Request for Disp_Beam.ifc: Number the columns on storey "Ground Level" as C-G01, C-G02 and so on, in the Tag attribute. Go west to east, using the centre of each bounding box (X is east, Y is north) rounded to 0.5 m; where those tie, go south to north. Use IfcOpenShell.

First a look at what the model holds.

```python
import ifcopenshell
import ifcopenshell.util.element
import ifcopenshell.util.placement

model = ifcopenshell.open("Disp_Beam.ifc")
print(model.schema)
storey = next(s for s in model.by_type("IfcBuildingStorey") if s.Name == "Ground Level")
columns = [e for e in ifcopenshell.util.element.get_decomposition(storey) if e.is_a("IfcColumn")]
for e in sorted(columns, key=lambda e: e.id()):
    origin = ifcopenshell.util.placement.get_local_placement(e.ObjectPlacement)[:3, 3]
    print(e.id(), e.Tag, e.Name, origin.round(2) + 0.0, sep=" | ")
```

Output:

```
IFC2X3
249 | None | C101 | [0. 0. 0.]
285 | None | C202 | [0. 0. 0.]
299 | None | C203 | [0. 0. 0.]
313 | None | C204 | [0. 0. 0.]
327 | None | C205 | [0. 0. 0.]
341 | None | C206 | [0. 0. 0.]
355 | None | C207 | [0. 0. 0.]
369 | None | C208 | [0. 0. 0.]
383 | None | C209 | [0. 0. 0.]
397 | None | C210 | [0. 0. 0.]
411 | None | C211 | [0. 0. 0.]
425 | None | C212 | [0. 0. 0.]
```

```python
import ifcopenshell
import ifcopenshell.geom
import ifcopenshell.util.element
import ifcopenshell.util.shape

model = ifcopenshell.open("Disp_Beam.ifc")
settings = ifcopenshell.geom.settings()
settings.set("use-world-coords", True)


def centre(element):
    shape = ifcopenshell.geom.create_shape(settings, element)
    return ifcopenshell.util.shape.get_bbox_centroid(shape.geometry)


storey = next(s for s in model.by_type("IfcBuildingStorey") if s.Name == "Ground Level")
columns = [e for e in ifcopenshell.util.element.get_decomposition(storey) if e.is_a("IfcColumn")]

# Insertion points can sit at a corner or the storey origin, so sort by the geometry (in metres).
centres = {e: centre(e) for e in columns}
columns.sort(key=lambda e: (round(centres[e][0] / 0.5), centres[e][1]))

for i, e in enumerate(columns, start=1):
    number = f"C-G{i:02d}"
    e.Tag = number
    print(e.id(), number)

model.write("Disp_Beam_v2.ifc")
```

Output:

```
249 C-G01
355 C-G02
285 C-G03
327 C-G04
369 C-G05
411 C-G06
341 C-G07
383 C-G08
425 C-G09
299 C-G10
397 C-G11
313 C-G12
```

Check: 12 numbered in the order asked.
